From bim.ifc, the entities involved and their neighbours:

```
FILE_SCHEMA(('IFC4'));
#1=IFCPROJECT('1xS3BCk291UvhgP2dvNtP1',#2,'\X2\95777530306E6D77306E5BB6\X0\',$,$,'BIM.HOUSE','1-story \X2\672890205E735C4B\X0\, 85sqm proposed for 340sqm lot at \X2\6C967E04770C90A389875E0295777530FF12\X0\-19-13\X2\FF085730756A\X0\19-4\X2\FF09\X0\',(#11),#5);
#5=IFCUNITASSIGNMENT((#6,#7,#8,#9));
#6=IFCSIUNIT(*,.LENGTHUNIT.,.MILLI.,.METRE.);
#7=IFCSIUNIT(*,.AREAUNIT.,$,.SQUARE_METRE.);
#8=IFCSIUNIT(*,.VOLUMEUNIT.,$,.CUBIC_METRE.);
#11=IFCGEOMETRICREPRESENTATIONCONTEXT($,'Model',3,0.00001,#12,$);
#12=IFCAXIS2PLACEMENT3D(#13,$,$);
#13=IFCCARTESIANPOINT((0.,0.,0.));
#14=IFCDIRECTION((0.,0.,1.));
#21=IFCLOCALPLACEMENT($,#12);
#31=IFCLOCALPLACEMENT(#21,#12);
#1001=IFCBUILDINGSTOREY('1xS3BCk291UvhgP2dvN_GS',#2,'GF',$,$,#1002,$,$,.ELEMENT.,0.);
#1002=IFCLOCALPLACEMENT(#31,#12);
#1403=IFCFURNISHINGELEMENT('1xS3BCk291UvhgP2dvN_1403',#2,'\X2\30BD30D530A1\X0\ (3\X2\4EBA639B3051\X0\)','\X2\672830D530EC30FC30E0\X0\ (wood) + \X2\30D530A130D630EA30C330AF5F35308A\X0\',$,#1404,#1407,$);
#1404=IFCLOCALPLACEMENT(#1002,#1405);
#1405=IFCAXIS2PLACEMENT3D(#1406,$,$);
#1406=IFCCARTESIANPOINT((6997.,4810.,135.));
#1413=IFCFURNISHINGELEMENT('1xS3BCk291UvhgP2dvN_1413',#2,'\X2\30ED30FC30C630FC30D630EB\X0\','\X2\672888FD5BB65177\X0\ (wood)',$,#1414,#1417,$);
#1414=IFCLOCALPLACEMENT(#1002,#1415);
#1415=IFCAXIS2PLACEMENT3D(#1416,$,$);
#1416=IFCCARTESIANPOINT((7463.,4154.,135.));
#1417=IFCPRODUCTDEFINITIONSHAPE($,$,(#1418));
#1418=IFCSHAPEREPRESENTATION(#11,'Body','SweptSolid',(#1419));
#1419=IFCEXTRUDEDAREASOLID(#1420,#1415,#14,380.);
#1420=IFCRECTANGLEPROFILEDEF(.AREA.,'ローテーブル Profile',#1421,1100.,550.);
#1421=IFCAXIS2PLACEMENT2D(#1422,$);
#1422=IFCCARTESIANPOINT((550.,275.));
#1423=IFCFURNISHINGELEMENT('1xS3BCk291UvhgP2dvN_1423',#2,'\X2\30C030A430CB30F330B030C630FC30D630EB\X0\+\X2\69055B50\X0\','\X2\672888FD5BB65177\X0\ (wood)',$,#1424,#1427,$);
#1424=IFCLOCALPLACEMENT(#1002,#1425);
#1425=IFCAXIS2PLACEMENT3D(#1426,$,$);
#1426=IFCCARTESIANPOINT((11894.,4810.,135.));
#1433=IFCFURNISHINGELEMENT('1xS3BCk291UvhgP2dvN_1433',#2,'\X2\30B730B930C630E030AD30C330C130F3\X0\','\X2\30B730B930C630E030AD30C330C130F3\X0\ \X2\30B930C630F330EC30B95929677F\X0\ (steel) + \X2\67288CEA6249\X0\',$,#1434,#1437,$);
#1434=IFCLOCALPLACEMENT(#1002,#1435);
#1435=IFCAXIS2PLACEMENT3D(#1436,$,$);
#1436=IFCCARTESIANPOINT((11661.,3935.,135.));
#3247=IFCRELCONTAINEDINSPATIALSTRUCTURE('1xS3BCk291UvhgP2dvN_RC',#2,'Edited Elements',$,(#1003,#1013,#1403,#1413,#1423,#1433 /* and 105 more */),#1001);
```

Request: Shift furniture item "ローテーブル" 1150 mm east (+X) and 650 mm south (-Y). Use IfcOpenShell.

```python
import ifcopenshell
import ifcopenshell.api.geometry
import ifcopenshell.util.placement
import ifcopenshell.util.unit

model = ifcopenshell.open("bim.ifc")
unit_scale = ifcopenshell.util.unit.calculate_unit_scale(model)

item = model.by_guid("1xS3BCk291UvhgP2dvN_1413")
matrix = ifcopenshell.util.placement.get_local_placement(item.ObjectPlacement)
matrix[0, 3] += 1.15 / unit_scale
matrix[1, 3] -= 0.65 / unit_scale
ifcopenshell.api.geometry.edit_object_placement(model, product=item, matrix=matrix, is_si=False)

print(ifcopenshell.util.placement.get_local_placement(item.ObjectPlacement).round(3) + 0.0)

model.write("bim_rev.ifc")
```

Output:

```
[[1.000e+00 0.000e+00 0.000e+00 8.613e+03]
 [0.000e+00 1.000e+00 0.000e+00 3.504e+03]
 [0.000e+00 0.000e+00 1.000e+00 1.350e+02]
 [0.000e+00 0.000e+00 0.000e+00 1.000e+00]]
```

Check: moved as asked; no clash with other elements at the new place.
